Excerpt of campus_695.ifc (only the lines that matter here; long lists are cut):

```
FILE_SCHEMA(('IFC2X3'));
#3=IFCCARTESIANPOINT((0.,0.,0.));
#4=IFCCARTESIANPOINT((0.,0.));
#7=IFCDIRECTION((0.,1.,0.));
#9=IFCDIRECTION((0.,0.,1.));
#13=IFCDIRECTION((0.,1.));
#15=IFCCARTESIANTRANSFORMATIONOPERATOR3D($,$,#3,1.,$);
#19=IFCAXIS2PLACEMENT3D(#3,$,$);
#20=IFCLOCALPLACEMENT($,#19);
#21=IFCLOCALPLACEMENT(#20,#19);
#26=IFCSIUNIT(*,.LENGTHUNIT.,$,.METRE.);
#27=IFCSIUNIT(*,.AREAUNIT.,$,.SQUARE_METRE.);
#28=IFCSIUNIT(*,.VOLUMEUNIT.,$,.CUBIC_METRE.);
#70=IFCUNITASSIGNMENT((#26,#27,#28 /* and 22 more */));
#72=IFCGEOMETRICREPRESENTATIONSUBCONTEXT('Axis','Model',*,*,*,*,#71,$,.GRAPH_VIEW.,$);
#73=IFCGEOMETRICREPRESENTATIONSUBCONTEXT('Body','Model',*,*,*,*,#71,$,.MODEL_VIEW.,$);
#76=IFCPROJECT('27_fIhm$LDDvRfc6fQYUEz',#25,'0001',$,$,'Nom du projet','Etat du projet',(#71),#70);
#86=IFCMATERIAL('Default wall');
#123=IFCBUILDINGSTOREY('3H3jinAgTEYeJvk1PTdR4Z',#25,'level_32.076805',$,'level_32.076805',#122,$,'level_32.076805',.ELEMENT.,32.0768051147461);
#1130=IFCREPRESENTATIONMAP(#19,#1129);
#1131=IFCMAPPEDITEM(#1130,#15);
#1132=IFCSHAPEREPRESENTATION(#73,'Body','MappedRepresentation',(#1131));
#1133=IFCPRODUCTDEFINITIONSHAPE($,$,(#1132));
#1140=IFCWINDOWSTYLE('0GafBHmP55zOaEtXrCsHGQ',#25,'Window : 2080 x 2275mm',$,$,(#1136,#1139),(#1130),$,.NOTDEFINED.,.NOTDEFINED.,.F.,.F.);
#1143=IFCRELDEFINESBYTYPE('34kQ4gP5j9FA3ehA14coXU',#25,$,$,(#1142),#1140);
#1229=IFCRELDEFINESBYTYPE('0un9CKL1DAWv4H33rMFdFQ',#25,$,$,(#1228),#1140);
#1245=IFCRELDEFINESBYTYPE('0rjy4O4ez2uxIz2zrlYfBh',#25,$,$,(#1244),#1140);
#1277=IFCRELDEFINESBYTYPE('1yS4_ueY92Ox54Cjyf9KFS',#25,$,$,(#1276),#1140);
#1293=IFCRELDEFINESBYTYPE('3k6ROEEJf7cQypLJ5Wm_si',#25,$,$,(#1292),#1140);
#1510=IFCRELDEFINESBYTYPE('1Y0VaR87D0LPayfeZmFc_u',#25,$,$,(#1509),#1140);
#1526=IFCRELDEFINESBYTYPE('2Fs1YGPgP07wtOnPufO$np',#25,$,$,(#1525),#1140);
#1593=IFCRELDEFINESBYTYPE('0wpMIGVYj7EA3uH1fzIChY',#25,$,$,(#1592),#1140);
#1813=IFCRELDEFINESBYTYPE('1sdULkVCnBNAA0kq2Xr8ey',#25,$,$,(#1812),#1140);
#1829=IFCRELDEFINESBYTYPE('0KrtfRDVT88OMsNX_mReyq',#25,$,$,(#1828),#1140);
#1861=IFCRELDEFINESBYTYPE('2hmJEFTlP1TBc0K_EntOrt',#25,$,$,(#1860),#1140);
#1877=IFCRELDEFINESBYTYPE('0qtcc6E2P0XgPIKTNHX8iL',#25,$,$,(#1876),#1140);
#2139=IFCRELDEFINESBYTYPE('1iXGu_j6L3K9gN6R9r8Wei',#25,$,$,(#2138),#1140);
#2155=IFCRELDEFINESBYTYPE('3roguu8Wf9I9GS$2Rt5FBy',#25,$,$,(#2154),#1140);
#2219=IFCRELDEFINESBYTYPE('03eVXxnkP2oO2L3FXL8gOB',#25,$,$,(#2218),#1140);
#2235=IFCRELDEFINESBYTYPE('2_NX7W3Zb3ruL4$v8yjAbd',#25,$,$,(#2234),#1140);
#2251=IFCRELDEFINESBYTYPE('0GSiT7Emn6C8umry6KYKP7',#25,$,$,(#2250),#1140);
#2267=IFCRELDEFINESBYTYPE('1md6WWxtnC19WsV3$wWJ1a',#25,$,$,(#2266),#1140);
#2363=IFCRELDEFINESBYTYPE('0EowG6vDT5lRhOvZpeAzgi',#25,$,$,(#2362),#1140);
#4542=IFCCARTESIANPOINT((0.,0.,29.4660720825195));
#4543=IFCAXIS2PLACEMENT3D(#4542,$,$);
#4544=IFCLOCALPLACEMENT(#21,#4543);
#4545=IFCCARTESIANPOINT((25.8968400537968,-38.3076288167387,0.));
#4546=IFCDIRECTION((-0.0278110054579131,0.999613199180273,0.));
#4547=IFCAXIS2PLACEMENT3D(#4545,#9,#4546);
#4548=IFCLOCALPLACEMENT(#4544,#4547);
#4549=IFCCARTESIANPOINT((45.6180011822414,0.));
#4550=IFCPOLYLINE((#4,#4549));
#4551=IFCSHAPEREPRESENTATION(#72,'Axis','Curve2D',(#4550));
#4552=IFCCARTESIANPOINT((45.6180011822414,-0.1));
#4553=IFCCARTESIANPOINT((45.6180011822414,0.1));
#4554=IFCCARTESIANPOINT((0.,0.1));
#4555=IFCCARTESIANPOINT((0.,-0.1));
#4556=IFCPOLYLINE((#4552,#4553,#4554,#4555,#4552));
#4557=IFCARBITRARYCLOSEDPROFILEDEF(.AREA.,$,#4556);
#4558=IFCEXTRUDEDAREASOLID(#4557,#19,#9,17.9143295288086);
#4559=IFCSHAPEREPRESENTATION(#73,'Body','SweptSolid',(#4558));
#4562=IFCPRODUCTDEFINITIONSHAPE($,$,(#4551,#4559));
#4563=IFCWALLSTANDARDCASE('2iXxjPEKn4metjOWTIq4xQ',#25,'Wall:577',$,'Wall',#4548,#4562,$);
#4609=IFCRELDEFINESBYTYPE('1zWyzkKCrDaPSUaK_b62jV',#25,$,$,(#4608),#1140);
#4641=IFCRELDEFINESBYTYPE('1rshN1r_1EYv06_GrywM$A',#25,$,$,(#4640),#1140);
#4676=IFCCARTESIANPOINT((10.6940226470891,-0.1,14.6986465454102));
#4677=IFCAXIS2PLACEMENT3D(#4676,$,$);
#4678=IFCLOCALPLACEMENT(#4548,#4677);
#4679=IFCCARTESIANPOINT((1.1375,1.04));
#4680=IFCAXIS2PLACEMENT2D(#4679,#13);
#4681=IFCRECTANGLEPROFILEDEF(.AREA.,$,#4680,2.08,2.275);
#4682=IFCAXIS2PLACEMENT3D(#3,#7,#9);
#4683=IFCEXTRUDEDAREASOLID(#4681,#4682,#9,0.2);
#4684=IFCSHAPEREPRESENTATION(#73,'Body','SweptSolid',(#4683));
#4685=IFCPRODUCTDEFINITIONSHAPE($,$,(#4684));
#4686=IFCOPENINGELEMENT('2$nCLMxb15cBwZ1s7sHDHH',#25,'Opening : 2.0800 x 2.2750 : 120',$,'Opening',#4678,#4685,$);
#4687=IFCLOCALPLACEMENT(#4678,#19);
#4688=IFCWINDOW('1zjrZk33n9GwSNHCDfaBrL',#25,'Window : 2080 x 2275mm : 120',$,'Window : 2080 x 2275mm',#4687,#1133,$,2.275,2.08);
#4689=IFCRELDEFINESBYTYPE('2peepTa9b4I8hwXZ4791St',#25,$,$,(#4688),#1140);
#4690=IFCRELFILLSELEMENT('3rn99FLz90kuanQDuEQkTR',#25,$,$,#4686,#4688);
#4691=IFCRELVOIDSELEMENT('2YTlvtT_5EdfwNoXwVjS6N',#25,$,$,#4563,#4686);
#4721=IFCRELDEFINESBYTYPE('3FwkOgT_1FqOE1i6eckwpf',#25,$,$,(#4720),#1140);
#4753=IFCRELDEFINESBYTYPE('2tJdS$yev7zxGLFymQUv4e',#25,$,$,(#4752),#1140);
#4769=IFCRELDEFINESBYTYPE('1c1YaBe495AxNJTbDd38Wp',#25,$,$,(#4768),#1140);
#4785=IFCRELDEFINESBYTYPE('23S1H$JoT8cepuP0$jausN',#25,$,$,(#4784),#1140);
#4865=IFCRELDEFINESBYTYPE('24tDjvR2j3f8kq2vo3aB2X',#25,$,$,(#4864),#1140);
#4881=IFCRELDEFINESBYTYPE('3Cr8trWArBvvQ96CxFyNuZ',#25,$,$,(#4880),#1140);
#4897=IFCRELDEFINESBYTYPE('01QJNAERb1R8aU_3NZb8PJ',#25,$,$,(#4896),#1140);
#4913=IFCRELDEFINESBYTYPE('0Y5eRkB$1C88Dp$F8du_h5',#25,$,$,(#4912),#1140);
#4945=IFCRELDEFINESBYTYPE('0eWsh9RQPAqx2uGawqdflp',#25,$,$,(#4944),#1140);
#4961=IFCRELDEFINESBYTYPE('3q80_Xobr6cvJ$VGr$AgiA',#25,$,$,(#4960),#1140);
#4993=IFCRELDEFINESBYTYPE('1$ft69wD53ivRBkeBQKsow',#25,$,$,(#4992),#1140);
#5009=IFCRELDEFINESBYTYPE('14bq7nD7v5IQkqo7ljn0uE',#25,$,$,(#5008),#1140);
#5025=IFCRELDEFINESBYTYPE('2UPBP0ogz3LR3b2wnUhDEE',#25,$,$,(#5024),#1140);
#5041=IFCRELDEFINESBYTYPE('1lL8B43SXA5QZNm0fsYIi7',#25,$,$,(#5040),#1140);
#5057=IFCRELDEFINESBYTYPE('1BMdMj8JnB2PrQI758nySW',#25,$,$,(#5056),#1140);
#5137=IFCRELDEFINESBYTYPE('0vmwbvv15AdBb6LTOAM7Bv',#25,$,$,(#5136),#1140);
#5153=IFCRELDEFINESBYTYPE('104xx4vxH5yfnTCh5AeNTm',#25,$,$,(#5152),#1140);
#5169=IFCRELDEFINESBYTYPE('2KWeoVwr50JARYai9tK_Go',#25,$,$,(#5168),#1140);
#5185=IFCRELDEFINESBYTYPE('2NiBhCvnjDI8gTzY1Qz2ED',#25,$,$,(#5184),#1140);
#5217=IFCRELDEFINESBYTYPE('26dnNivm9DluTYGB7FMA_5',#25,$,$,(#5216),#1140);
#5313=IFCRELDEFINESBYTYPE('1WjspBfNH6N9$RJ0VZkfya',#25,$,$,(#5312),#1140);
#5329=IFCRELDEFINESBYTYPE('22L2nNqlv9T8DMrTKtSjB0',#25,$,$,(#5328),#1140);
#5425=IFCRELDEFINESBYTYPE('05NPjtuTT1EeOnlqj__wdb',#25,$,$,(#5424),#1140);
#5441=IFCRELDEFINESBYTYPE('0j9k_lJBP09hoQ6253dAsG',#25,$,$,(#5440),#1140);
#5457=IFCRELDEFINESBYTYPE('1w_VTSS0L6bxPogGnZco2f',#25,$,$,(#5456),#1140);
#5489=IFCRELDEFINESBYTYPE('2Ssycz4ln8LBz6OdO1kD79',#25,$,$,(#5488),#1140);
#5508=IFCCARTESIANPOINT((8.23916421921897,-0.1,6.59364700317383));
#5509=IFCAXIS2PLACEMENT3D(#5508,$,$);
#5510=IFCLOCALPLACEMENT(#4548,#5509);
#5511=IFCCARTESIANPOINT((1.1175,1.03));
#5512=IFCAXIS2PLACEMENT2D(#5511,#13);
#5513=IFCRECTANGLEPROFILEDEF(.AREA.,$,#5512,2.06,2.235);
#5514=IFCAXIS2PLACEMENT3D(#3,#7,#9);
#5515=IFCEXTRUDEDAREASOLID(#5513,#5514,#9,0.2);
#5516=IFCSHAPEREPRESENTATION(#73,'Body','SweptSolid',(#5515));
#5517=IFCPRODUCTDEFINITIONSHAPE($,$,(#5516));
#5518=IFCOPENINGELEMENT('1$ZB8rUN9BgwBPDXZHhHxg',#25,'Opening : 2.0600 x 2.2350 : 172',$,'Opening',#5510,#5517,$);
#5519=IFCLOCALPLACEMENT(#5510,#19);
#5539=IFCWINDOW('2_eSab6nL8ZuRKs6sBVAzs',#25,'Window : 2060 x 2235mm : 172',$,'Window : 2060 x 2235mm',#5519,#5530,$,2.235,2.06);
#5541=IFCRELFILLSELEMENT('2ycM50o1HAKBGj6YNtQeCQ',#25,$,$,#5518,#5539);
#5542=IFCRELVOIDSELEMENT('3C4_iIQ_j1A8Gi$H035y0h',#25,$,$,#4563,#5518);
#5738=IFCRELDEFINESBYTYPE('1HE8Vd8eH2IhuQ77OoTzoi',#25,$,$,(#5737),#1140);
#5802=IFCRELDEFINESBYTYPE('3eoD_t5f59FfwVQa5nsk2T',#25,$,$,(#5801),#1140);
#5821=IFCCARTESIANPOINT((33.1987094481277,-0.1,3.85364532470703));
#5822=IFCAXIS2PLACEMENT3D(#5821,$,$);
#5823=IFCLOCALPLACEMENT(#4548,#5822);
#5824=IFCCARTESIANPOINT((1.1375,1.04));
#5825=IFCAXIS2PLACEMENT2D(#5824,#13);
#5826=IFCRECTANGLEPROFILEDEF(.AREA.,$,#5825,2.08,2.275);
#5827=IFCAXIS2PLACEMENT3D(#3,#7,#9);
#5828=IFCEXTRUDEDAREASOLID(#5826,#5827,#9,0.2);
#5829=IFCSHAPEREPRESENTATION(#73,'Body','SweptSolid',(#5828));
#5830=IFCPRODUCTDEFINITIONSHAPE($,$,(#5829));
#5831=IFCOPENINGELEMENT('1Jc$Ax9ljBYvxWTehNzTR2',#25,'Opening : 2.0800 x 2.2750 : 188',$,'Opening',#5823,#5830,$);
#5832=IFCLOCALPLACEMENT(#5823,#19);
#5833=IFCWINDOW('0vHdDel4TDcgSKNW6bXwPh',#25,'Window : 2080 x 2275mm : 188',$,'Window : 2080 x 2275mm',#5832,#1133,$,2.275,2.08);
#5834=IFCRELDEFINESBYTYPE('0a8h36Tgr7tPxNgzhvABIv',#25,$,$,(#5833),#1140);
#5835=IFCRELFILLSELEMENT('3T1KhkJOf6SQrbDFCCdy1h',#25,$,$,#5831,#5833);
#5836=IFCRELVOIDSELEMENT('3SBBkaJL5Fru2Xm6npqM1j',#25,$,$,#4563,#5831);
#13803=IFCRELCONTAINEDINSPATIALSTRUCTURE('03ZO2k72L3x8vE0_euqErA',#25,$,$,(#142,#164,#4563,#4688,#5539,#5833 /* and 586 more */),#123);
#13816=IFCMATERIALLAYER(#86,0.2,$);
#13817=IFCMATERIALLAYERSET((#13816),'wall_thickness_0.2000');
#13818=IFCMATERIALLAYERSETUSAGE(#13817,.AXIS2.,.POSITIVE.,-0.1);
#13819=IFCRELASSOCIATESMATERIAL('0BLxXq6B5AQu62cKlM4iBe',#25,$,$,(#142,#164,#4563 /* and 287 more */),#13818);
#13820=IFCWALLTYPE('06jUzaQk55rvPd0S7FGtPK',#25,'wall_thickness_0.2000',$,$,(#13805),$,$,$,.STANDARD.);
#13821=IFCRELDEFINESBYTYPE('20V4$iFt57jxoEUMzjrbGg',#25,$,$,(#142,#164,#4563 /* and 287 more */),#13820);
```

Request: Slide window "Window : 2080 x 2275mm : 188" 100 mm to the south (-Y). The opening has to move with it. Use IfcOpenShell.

```python
import ifcopenshell
import ifcopenshell.api.geometry
import ifcopenshell.util.placement
import ifcopenshell.util.unit

model = ifcopenshell.open("campus_695.ifc")
unit_scale = ifcopenshell.util.unit.calculate_unit_scale(model)

window = model.by_guid("0vHdDel4TDcgSKNW6bXwPh")
opening = window.FillsVoids[0].RelatingOpeningElement
wall = opening.VoidsElements[0].RelatingBuildingElement

wall_matrix = ifcopenshell.util.placement.get_local_placement(wall.ObjectPlacement)
shift = wall_matrix[:3, 0] * -0.1 / unit_scale
before = ifcopenshell.util.placement.get_local_placement(window.ObjectPlacement)[:3, 3].copy()

# The window is placed relative to its opening, so it follows when the opening moves.
matrix = ifcopenshell.util.placement.get_local_placement(opening.ObjectPlacement)
matrix[:3, 3] += shift
ifcopenshell.api.geometry.edit_object_placement(
    model, product=opening, matrix=matrix, is_si=False, should_transform_children=True
)

after = ifcopenshell.util.placement.get_local_placement(window.ObjectPlacement)[:3, 3]
print("window moved by", (after - before).round(3) + 0.0)

model.write("campus_695_edited.ifc")
```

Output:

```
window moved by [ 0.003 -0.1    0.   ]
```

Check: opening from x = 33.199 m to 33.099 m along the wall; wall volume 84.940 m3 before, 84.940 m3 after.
